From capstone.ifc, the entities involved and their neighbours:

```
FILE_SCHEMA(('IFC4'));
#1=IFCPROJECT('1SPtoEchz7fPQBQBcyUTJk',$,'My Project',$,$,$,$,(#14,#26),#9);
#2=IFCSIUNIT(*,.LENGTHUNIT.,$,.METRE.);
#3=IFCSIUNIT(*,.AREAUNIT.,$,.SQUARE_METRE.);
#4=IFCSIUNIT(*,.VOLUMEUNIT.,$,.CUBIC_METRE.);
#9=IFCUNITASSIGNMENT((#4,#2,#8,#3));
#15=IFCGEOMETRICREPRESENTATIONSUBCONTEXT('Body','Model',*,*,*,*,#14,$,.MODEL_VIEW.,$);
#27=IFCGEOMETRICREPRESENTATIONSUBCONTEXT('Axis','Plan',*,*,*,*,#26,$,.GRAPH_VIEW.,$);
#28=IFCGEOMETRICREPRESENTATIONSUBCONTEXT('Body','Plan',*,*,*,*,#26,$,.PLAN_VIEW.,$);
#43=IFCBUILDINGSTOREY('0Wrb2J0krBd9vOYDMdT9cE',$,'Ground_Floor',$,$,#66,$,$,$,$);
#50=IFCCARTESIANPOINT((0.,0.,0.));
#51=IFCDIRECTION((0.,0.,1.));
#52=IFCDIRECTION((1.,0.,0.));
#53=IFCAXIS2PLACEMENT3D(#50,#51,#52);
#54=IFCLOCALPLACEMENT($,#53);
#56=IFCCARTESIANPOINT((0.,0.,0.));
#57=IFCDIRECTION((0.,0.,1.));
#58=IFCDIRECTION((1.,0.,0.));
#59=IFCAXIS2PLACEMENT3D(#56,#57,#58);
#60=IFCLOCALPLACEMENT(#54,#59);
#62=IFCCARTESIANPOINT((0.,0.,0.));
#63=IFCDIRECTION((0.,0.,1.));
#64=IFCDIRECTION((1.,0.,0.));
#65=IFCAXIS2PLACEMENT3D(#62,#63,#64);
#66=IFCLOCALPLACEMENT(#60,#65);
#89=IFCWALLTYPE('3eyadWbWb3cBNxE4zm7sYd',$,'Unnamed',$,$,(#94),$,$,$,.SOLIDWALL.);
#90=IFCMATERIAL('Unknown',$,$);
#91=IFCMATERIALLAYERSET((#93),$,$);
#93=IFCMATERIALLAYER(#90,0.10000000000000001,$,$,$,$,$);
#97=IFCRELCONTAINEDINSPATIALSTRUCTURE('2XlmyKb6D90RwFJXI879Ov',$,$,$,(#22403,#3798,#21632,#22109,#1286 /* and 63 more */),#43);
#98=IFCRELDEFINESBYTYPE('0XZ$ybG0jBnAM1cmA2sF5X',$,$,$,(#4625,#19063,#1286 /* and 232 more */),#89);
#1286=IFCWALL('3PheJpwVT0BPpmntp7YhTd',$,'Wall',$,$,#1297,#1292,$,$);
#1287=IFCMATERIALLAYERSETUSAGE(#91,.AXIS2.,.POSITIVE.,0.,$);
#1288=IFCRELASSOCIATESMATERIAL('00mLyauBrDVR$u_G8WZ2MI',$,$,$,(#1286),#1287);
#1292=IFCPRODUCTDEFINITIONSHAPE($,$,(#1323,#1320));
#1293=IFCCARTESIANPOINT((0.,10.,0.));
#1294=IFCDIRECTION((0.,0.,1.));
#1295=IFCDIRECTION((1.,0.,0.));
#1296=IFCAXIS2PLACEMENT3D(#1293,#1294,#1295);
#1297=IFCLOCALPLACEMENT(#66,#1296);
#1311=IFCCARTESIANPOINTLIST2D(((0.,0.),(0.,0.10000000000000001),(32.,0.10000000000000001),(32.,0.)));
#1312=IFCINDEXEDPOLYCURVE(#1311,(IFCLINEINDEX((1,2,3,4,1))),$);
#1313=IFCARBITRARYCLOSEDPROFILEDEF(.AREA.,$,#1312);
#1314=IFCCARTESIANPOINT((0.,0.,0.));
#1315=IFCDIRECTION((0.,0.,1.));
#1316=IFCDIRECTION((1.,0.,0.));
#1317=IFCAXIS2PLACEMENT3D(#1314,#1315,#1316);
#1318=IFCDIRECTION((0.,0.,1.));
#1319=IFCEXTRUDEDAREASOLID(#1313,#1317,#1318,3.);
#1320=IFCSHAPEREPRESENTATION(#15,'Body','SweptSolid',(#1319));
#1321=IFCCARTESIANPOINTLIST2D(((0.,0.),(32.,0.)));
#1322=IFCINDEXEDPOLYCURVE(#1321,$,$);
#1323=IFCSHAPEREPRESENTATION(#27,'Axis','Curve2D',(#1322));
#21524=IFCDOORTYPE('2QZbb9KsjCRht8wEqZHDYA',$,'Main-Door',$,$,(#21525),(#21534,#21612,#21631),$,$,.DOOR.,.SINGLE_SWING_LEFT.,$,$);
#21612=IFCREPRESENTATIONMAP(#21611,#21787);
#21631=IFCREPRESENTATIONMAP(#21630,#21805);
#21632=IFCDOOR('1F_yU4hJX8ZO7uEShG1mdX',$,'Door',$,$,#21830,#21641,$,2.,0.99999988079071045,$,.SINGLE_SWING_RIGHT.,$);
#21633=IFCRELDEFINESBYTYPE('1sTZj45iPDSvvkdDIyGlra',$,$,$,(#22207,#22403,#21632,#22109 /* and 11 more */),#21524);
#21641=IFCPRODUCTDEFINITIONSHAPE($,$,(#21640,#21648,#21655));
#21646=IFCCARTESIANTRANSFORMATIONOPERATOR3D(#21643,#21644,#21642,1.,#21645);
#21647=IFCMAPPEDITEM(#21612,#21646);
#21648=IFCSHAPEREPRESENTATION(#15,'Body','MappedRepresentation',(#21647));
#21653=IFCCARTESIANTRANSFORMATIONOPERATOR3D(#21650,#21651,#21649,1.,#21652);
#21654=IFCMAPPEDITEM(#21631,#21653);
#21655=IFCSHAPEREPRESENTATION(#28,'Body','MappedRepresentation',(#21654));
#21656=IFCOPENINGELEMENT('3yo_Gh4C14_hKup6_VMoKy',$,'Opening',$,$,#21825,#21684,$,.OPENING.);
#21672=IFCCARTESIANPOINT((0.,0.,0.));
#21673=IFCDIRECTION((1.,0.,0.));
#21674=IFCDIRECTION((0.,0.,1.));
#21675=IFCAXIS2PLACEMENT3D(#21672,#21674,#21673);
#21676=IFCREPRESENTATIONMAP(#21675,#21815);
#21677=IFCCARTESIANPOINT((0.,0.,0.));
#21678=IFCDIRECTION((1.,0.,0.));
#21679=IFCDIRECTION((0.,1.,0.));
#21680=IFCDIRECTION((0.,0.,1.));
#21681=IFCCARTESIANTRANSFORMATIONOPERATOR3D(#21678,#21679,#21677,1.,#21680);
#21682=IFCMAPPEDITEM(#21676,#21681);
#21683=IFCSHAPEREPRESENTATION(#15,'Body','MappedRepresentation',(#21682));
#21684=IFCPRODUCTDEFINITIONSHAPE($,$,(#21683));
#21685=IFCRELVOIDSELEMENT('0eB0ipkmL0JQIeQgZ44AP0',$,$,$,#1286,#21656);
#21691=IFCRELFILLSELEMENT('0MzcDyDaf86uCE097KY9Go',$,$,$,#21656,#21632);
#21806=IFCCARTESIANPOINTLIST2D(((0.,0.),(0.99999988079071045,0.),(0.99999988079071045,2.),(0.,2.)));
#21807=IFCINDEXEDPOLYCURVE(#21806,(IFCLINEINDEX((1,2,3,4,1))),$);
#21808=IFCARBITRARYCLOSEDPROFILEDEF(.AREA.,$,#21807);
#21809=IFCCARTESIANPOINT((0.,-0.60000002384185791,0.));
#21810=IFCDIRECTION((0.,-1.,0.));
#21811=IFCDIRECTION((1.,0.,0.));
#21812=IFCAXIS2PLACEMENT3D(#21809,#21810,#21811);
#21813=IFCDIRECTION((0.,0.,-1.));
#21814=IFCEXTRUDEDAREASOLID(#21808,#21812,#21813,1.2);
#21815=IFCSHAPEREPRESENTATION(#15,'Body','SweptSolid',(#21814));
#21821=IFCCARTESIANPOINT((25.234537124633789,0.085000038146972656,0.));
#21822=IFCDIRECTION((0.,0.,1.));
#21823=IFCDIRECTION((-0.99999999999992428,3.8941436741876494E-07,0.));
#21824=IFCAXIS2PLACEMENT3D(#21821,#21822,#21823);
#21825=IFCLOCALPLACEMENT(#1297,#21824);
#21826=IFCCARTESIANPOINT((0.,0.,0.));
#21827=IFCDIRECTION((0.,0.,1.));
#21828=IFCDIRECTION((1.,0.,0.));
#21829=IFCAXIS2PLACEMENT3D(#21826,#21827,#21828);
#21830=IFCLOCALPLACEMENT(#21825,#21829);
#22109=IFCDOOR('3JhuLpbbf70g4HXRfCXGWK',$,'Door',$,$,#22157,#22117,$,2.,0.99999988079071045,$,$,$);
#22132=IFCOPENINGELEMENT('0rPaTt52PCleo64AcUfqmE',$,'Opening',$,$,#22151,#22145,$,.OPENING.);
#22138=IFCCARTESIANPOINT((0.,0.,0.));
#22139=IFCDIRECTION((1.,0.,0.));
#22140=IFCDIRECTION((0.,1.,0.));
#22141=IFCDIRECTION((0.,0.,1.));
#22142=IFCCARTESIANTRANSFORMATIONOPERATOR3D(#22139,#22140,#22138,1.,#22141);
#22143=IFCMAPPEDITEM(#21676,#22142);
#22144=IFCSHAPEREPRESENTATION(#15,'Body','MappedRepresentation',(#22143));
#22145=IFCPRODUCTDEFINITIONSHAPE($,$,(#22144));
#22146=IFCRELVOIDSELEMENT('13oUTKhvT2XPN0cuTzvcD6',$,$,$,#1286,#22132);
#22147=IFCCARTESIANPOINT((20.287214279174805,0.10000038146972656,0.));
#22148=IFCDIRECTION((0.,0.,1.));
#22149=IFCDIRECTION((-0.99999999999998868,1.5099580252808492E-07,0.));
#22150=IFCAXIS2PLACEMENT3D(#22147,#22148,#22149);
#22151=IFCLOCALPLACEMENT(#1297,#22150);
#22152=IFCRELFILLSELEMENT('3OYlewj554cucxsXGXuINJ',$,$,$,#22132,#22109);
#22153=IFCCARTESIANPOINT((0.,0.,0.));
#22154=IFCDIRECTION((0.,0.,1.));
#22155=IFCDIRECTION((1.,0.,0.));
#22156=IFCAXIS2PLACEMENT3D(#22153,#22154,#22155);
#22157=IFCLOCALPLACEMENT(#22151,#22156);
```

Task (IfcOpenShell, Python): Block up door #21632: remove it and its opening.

```python
import ifcopenshell
import ifcopenshell.api.feature
import ifcopenshell.api.root
import ifcopenshell.geom
import ifcopenshell.util.shape

model = ifcopenshell.open("capstone.ifc")
settings = ifcopenshell.geom.settings()


def volume(element):
    """Net volume in cubic metres, openings subtracted."""
    shape = ifcopenshell.geom.create_shape(settings, element)
    return ifcopenshell.util.shape.get_volume(shape.geometry)


door = model.by_guid("1F_yU4hJX8ZO7uEShG1mdX")
opening = door.FillsVoids[0].RelatingOpeningElement
wall = opening.VoidsElements[0].RelatingBuildingElement
before = volume(wall)

ifcopenshell.api.root.remove_product(model, product=door)
ifcopenshell.api.feature.remove_feature(model, feature=opening)

after = volume(wall)

print(f"wall volume {before:.3f} -> {after:.3f} m3")

model.write("capstone_v2.ifc")
```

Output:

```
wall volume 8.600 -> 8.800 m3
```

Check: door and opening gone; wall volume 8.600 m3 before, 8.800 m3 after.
